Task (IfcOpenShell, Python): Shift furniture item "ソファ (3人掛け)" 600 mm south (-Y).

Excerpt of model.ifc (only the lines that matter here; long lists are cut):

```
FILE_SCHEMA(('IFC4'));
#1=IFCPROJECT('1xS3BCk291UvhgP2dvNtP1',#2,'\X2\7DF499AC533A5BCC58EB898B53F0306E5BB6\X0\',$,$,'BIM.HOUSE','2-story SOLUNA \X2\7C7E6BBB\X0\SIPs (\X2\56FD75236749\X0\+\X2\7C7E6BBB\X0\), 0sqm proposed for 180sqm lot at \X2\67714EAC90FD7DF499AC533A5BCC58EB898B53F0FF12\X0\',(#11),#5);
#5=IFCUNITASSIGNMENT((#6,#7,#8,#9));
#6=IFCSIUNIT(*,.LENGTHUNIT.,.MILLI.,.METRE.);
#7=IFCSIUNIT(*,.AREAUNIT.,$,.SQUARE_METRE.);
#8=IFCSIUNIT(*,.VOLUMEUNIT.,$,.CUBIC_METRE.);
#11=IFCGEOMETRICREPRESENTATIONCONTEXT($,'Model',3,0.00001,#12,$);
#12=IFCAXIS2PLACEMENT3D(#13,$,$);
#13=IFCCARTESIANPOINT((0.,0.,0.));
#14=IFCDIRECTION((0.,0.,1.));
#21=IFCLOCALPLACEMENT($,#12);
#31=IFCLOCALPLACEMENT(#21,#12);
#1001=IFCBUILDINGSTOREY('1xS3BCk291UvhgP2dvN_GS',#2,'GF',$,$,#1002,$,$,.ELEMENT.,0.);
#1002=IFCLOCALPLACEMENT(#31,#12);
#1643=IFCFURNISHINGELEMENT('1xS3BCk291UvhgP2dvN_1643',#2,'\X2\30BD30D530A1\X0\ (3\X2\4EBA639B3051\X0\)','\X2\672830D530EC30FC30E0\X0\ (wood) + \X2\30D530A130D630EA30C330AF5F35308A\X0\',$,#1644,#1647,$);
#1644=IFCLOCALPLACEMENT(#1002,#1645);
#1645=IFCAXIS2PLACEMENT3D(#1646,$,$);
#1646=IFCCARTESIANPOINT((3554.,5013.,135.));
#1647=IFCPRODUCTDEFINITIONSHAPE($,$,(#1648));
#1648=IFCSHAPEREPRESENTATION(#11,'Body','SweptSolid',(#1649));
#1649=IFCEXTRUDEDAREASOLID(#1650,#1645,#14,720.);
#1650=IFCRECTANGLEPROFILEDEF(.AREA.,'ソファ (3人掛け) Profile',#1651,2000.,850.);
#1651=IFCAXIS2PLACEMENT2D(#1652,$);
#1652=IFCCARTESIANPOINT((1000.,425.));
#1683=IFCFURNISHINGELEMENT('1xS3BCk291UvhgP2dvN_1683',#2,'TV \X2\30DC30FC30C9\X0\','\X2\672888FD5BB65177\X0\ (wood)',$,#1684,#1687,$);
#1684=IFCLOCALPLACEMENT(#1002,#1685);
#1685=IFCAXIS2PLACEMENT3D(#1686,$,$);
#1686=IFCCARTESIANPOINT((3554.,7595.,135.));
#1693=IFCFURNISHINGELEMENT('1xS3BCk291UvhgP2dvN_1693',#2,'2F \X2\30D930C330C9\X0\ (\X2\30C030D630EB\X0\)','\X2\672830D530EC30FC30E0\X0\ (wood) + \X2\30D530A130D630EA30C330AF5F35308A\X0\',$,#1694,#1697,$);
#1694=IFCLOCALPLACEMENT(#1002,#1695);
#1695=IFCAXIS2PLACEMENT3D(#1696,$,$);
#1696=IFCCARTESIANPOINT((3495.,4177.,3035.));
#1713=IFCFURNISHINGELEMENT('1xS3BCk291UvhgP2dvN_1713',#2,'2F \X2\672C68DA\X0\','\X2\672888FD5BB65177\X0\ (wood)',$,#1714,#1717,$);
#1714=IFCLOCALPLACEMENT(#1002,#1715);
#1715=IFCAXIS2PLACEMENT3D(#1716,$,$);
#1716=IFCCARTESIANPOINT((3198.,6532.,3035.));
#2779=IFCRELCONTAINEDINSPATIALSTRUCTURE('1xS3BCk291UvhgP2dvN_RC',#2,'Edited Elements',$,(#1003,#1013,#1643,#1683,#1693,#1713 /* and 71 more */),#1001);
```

```python
import ifcopenshell
import ifcopenshell.api.geometry
import ifcopenshell.util.placement
import ifcopenshell.util.unit

model = ifcopenshell.open("model.ifc")
unit_scale = ifcopenshell.util.unit.calculate_unit_scale(model)

item = model.by_guid("1xS3BCk291UvhgP2dvN_1643")
matrix = ifcopenshell.util.placement.get_local_placement(item.ObjectPlacement)
matrix[1, 3] -= 0.6 / unit_scale
ifcopenshell.api.geometry.edit_object_placement(model, product=item, matrix=matrix, is_si=False)

print(ifcopenshell.util.placement.get_local_placement(item.ObjectPlacement).round(3) + 0.0)

model.write("model_edited.ifc")
```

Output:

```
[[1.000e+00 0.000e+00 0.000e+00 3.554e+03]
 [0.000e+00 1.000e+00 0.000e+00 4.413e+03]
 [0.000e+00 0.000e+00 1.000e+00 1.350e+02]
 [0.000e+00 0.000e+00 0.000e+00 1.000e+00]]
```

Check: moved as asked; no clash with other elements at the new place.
